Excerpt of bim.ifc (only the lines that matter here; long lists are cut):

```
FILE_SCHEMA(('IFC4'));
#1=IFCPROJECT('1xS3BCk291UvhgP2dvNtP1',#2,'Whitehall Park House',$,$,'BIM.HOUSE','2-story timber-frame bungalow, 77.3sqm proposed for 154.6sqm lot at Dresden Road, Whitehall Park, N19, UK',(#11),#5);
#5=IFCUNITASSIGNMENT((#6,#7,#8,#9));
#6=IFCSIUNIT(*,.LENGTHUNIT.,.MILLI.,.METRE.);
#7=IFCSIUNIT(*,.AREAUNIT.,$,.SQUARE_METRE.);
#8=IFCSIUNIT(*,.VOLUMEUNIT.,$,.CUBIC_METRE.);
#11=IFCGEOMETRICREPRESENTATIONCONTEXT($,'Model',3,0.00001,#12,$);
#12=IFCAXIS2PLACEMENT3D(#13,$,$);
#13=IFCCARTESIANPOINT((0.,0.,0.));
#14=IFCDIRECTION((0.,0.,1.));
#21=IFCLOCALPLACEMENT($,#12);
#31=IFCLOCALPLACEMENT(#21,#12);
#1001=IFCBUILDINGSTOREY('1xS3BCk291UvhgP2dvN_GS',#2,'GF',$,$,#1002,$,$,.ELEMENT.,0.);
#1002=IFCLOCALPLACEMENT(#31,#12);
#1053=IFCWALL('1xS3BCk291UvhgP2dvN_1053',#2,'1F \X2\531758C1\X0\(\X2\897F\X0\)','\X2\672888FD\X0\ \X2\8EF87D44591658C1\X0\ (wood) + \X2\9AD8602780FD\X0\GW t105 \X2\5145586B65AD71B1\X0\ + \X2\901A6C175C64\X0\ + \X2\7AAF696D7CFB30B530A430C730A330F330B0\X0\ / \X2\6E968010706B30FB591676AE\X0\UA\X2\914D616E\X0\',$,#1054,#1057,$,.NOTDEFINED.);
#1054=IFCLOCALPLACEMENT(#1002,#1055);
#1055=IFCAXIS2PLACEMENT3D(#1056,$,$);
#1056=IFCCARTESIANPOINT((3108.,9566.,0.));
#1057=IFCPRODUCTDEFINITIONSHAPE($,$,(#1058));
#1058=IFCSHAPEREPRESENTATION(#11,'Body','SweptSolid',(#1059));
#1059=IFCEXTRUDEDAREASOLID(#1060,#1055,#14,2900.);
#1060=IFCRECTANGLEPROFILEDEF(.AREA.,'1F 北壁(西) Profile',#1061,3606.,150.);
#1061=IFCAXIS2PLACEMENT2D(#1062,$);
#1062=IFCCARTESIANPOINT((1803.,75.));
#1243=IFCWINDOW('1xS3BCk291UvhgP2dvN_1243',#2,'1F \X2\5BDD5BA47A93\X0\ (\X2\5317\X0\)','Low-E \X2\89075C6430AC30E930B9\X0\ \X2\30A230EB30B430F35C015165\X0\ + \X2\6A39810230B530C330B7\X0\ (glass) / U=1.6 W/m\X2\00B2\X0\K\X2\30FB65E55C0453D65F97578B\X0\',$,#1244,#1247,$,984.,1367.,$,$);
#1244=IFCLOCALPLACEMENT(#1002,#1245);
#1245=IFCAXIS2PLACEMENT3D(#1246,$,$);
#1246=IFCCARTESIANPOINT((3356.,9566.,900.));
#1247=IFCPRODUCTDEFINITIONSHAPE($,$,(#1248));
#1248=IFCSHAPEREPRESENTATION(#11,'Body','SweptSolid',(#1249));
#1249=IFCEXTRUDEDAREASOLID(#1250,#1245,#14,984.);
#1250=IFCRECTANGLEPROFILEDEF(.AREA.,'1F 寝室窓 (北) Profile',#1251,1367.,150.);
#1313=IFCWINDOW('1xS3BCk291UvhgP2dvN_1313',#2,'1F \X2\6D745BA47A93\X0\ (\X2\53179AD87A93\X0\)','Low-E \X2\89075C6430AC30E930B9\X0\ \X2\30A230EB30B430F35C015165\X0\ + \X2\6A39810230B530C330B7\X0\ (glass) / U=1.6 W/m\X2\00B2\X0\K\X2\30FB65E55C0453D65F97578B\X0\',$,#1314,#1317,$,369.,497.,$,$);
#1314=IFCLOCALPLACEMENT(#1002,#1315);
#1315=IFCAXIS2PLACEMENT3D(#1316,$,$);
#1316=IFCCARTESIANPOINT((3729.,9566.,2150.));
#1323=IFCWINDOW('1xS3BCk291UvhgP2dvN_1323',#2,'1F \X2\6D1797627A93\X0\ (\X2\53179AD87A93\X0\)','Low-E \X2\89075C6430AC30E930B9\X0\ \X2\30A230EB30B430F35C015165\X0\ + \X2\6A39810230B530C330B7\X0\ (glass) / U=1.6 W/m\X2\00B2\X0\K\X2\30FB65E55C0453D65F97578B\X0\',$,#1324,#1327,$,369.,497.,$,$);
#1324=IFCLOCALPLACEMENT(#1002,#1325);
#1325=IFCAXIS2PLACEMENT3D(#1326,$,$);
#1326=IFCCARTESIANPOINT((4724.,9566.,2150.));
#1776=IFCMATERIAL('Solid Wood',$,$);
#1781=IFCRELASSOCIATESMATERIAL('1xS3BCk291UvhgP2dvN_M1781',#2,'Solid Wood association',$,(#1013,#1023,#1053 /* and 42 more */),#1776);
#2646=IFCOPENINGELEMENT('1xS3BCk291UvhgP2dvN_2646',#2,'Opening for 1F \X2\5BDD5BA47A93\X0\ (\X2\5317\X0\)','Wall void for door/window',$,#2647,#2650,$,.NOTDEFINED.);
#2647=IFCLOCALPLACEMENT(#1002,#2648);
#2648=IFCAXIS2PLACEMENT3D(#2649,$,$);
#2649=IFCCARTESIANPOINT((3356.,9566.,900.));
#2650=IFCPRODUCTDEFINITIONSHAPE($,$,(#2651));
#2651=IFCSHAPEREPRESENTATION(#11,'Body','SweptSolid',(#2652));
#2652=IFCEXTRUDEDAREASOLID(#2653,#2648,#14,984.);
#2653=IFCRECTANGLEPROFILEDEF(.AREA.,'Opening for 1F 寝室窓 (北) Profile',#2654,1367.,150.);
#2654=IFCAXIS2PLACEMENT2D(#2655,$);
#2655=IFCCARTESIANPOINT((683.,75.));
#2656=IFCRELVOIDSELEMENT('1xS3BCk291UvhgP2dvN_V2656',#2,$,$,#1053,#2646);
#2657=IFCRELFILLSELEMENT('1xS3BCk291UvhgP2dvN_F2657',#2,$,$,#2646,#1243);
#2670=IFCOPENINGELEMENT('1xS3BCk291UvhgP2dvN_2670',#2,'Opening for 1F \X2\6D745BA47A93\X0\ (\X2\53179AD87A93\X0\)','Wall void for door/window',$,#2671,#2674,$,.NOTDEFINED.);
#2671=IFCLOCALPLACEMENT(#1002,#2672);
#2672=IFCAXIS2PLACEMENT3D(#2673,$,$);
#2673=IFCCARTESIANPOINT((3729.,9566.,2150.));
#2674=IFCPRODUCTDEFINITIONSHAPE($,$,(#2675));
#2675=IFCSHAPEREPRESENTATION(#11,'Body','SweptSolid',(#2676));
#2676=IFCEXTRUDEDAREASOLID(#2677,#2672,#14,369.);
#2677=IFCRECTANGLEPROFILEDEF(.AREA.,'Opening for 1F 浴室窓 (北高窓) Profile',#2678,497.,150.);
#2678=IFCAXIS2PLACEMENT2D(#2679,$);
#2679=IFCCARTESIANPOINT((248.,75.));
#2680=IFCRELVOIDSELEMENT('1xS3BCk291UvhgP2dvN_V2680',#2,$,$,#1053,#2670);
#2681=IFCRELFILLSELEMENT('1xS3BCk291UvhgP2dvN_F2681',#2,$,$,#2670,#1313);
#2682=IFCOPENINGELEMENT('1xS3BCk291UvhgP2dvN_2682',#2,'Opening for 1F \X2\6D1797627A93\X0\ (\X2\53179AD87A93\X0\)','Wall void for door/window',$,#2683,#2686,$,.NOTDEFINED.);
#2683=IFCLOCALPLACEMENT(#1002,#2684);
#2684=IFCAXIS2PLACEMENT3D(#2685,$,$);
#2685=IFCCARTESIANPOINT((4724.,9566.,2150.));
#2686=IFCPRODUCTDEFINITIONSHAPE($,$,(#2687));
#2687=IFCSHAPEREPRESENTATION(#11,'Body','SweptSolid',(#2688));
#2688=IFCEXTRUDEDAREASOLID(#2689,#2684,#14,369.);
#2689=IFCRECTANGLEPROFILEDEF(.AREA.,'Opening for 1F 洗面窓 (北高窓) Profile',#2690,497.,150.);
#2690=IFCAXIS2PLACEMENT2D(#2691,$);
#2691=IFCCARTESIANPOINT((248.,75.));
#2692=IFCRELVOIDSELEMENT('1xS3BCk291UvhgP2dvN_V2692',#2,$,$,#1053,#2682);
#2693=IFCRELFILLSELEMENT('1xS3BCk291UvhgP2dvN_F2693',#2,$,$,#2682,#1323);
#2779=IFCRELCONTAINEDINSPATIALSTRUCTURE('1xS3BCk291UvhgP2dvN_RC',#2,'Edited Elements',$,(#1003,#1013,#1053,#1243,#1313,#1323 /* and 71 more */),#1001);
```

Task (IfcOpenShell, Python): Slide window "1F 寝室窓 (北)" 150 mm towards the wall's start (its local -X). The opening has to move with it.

```python
import ifcopenshell
import ifcopenshell.api.geometry
import ifcopenshell.util.placement
import ifcopenshell.util.unit

model = ifcopenshell.open("bim.ifc")
unit_scale = ifcopenshell.util.unit.calculate_unit_scale(model)

window = model.by_id(1243)
opening = window.FillsVoids[0].RelatingOpeningElement
wall = opening.VoidsElements[0].RelatingBuildingElement

wall_matrix = ifcopenshell.util.placement.get_local_placement(wall.ObjectPlacement)
shift = wall_matrix[:3, 0] * -0.15 / unit_scale
before = ifcopenshell.util.placement.get_local_placement(window.ObjectPlacement)[:3, 3].copy()

# The window is not placed relative to its opening, so move both.
for product in (opening, window):
    matrix = ifcopenshell.util.placement.get_local_placement(product.ObjectPlacement)
    matrix[:3, 3] += shift
    ifcopenshell.api.geometry.edit_object_placement(model, product=product, matrix=matrix, is_si=False)

after = ifcopenshell.util.placement.get_local_placement(window.ObjectPlacement)[:3, 3]
print("window moved by", (after - before).round(3) + 0.0)

model.write("bim_updated.ifc")
```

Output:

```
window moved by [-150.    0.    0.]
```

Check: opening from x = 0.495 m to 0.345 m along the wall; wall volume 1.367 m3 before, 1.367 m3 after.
